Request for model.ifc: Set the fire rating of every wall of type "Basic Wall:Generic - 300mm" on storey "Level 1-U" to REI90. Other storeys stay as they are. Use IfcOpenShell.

First a look at what the model holds.

```python
import ifcopenshell
import ifcopenshell.util.element

model = ifcopenshell.open("model.ifc")
print(model.schema)
storey = next(s for s in model.by_type("IfcBuildingStorey") if s.Name == "Level 1-U")
walls = [e for e in ifcopenshell.util.element.get_decomposition(storey) if e.is_a("IfcWall")]
seen = {}
for e in walls:
    element_type = ifcopenshell.util.element.get_type(e)
    key = (element_type.Name if element_type != e and element_type else None, ifcopenshell.util.element.get_pset(e, "Pset_WallCommon", "FireRating"))
    seen[key] = seen.get(key, 0) + 1
for (name, value), count in sorted(seen.items(), key=str):
    print(count, "x", name, "|", value)
```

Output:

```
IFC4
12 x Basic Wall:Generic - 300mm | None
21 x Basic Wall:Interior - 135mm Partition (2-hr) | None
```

```python
import ifcopenshell
import ifcopenshell.api.pset
import ifcopenshell.util.element

model = ifcopenshell.open("model.ifc")

storey = next(s for s in model.by_type("IfcBuildingStorey") if s.Name == "Level 1-U")
walls = [e for e in ifcopenshell.util.element.get_decomposition(storey) if e.is_a("IfcWall")]

count = 0
for e in walls:
    element_type = ifcopenshell.util.element.get_type(e)
    if element_type in (None, e) or element_type.Name != "Basic Wall:Generic - 300mm":
        continue
    # add_pset returns the element's existing set when there is one.
    pset = ifcopenshell.api.pset.add_pset(model, product=e, name="Pset_WallCommon")
    ifcopenshell.api.pset.edit_pset(model, pset=pset, properties={"FireRating": "REI90"})
    count += 1

print(count, "walls updated")

model.write("model-out.ifc")
```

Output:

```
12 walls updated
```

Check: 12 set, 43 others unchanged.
